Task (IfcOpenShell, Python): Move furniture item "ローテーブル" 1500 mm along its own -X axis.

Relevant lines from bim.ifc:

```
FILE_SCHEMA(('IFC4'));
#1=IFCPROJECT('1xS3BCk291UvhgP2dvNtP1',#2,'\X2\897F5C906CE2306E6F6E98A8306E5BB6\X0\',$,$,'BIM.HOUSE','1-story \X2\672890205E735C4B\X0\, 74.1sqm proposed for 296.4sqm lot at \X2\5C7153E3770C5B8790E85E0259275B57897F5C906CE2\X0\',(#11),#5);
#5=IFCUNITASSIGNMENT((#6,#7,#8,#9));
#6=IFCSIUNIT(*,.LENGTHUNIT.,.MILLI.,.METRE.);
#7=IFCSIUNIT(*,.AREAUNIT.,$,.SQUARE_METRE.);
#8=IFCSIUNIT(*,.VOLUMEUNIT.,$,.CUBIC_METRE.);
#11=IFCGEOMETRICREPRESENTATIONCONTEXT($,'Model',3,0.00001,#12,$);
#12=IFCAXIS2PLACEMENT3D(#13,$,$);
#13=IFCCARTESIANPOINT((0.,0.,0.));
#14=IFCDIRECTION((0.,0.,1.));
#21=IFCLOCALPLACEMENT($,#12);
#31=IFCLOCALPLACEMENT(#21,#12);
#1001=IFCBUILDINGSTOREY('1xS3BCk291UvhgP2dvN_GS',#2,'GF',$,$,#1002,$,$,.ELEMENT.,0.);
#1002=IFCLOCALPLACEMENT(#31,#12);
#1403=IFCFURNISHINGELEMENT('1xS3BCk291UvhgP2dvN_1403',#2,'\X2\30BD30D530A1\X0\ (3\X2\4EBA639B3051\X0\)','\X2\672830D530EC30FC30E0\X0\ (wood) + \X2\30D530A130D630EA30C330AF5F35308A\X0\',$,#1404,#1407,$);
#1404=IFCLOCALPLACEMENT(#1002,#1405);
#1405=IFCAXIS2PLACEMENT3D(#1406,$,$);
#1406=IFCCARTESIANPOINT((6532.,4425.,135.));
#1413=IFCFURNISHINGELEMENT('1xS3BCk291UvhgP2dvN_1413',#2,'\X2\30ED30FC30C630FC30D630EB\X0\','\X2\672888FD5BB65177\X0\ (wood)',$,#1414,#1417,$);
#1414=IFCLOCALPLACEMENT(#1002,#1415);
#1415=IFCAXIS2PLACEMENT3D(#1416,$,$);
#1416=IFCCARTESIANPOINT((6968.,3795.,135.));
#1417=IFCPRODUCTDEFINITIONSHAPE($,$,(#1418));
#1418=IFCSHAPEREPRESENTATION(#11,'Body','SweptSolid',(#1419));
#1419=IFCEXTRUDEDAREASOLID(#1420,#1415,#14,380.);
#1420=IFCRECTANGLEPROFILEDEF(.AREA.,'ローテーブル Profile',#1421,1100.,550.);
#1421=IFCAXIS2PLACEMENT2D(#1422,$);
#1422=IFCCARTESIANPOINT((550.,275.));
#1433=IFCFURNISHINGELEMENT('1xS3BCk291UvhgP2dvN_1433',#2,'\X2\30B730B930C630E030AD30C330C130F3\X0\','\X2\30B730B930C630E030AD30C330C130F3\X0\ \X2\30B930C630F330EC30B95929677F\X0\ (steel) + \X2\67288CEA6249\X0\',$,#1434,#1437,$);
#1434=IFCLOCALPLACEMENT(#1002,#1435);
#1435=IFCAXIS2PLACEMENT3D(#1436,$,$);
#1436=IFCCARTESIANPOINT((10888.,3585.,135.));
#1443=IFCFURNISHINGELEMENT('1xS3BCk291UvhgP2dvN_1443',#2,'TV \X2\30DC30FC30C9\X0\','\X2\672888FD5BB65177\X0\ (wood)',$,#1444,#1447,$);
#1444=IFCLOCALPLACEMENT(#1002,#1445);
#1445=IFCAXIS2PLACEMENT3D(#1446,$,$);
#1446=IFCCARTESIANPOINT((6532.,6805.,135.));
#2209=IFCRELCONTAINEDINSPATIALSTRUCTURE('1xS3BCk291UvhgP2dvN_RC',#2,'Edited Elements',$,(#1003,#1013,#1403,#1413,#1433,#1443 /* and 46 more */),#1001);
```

```python
import ifcopenshell
import ifcopenshell.api.geometry
import ifcopenshell.util.placement
import ifcopenshell.util.unit

model = ifcopenshell.open("bim.ifc")
unit_scale = ifcopenshell.util.unit.calculate_unit_scale(model)

item = model.by_guid("1xS3BCk291UvhgP2dvN_1413")
matrix = ifcopenshell.util.placement.get_local_placement(item.ObjectPlacement)
matrix[:3, 3] -= matrix[:3, 0] * 1.5 / unit_scale
ifcopenshell.api.geometry.edit_object_placement(model, product=item, matrix=matrix, is_si=False)

print(ifcopenshell.util.placement.get_local_placement(item.ObjectPlacement).round(3) + 0.0)

model.write("bim-out.ifc")
```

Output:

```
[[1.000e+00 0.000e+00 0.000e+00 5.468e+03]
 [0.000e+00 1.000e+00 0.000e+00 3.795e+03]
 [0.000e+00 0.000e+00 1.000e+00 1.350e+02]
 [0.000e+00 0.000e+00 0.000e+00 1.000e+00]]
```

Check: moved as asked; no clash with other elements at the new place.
